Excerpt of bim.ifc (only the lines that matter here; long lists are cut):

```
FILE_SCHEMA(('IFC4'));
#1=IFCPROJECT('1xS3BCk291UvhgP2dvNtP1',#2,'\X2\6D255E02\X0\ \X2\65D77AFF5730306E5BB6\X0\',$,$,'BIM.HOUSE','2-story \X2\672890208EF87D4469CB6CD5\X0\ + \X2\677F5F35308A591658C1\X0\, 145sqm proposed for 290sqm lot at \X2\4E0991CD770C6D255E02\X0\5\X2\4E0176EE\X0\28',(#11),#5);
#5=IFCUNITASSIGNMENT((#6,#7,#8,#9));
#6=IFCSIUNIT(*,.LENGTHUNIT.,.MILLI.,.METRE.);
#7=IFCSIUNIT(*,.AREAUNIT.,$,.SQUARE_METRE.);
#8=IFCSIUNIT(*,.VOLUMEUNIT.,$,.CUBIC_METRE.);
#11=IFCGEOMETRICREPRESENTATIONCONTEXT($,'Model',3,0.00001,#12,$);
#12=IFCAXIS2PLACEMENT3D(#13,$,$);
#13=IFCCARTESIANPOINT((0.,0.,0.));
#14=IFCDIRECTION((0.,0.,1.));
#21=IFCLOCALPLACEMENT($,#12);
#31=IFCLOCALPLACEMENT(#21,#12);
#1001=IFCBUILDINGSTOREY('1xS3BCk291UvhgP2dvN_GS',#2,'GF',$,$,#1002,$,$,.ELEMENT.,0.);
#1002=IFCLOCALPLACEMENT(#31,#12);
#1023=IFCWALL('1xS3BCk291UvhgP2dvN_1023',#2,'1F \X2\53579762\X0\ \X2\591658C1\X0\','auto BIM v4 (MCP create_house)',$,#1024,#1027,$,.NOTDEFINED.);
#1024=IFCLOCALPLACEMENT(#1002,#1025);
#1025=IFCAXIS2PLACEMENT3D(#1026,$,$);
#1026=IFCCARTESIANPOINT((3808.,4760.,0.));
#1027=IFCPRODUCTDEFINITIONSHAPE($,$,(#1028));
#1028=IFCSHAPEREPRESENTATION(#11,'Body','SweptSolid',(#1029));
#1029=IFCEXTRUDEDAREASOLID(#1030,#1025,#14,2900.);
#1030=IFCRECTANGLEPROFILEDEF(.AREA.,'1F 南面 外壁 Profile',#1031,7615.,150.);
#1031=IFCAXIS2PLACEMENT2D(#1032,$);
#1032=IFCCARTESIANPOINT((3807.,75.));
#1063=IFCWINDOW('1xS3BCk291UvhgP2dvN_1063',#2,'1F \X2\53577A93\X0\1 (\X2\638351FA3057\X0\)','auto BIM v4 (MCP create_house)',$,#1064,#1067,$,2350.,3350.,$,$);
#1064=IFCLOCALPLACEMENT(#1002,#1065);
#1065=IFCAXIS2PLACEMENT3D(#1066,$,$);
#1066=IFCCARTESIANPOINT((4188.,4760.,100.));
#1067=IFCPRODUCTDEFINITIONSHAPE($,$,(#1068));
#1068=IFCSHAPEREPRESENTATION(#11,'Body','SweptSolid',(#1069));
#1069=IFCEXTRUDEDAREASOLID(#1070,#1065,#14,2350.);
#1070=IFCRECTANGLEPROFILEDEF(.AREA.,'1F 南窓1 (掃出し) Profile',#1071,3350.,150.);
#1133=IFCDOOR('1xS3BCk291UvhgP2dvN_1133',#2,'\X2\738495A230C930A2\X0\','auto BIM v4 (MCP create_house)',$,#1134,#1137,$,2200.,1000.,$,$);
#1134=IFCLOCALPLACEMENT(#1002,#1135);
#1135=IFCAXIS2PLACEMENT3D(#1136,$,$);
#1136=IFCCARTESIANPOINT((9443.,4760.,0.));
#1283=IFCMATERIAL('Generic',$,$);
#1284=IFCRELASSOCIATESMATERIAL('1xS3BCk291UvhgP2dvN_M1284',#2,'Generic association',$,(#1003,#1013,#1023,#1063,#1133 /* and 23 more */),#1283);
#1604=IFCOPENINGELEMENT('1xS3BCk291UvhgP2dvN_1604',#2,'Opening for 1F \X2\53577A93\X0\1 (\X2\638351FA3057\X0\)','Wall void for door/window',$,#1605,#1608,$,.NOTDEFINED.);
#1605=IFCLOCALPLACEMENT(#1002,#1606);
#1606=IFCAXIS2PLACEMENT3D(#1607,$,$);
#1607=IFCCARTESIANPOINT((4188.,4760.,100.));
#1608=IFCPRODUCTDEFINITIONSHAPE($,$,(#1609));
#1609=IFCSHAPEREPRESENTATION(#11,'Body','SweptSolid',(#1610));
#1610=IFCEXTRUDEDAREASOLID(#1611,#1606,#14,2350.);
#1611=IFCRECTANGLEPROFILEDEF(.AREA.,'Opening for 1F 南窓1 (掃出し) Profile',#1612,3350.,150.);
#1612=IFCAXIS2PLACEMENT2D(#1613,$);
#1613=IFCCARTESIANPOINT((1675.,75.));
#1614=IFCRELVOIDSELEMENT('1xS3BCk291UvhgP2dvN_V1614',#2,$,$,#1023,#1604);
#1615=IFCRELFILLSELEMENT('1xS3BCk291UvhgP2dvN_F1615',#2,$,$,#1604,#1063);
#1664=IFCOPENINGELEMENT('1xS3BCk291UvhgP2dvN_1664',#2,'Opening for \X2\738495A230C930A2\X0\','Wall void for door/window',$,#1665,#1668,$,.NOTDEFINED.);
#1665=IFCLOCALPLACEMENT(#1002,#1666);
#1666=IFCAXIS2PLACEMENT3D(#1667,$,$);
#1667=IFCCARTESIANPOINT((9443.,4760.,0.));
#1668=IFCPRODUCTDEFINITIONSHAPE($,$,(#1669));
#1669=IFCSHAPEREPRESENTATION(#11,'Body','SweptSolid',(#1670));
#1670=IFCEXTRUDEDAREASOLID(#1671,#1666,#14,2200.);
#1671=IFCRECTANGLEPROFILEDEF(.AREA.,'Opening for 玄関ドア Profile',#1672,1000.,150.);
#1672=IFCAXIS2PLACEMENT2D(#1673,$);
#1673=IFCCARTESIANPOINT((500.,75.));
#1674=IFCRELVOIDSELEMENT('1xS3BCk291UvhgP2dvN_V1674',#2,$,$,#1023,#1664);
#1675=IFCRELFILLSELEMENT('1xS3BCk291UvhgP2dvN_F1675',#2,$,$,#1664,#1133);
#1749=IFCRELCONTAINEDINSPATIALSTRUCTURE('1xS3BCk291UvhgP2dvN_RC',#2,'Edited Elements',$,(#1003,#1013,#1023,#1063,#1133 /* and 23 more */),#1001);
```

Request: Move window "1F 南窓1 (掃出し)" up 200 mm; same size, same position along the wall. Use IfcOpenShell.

```python
import numpy as np
import ifcopenshell
import ifcopenshell.api.geometry
import ifcopenshell.util.placement
import ifcopenshell.util.unit

model = ifcopenshell.open("bim.ifc")
unit_scale = ifcopenshell.util.unit.calculate_unit_scale(model)

window = model.by_guid("1xS3BCk291UvhgP2dvN_1063")
opening = window.FillsVoids[0].RelatingOpeningElement
dz = 0.2 / unit_scale

shift = np.array([0.0, 0.0, dz])
# The window is not placed relative to its opening, so move both.
for product in (opening, window):
    matrix = ifcopenshell.util.placement.get_local_placement(product.ObjectPlacement)
    matrix[:3, 3] += shift
    ifcopenshell.api.geometry.edit_object_placement(model, product=product, matrix=matrix, is_si=False)

print(f"moved by {dz * unit_scale:+.3f} m")

model.write("bim_updated.ifc")
```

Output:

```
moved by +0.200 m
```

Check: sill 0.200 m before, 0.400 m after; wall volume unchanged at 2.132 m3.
